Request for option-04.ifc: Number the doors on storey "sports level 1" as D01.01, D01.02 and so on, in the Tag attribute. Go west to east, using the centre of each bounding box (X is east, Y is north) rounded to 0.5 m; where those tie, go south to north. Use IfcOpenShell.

First a look at what the model holds.

```python
import ifcopenshell
import ifcopenshell.util.element
import ifcopenshell.util.placement

model = ifcopenshell.open("option-04.ifc")
print(model.schema)
storey = next(s for s in model.by_type("IfcBuildingStorey") if s.Name == "sports level 1")
doors = [e for e in ifcopenshell.util.element.get_decomposition(storey) if e.is_a("IfcDoor")]
for e in sorted(doors, key=lambda e: e.id()):
    origin = ifcopenshell.util.placement.get_local_placement(e.ObjectPlacement)[:3, 3]
    print(e.id(), e.Tag, e.Name, origin.round(2) + 0.0, sep=" | ")
```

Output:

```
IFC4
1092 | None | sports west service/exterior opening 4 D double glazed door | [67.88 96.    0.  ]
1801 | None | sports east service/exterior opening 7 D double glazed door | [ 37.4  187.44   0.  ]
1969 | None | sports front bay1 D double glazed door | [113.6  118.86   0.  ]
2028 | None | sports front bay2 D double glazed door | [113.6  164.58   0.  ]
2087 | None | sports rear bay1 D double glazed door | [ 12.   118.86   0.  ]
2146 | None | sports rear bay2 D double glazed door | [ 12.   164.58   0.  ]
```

```python
import ifcopenshell
import ifcopenshell.geom
import ifcopenshell.util.element
import ifcopenshell.util.shape

model = ifcopenshell.open("option-04.ifc")
settings = ifcopenshell.geom.settings()
settings.set("use-world-coords", True)


def centre(element):
    shape = ifcopenshell.geom.create_shape(settings, element)
    return ifcopenshell.util.shape.get_bbox_centroid(shape.geometry)


storey = next(s for s in model.by_type("IfcBuildingStorey") if s.Name == "sports level 1")
doors = [e for e in ifcopenshell.util.element.get_decomposition(storey) if e.is_a("IfcDoor")]

# Insertion points can sit at a corner or the storey origin, so sort by the geometry (in metres).
centres = {e: centre(e) for e in doors}
doors.sort(key=lambda e: (round(centres[e][0] / 0.5), centres[e][1]))

for i, e in enumerate(doors, start=1):
    number = f"D01.{i:02d}"
    e.Tag = number
    print(e.id(), number)

model.write("option-04_v2.ifc")
```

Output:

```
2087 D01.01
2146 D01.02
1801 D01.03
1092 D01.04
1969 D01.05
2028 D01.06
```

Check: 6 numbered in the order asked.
